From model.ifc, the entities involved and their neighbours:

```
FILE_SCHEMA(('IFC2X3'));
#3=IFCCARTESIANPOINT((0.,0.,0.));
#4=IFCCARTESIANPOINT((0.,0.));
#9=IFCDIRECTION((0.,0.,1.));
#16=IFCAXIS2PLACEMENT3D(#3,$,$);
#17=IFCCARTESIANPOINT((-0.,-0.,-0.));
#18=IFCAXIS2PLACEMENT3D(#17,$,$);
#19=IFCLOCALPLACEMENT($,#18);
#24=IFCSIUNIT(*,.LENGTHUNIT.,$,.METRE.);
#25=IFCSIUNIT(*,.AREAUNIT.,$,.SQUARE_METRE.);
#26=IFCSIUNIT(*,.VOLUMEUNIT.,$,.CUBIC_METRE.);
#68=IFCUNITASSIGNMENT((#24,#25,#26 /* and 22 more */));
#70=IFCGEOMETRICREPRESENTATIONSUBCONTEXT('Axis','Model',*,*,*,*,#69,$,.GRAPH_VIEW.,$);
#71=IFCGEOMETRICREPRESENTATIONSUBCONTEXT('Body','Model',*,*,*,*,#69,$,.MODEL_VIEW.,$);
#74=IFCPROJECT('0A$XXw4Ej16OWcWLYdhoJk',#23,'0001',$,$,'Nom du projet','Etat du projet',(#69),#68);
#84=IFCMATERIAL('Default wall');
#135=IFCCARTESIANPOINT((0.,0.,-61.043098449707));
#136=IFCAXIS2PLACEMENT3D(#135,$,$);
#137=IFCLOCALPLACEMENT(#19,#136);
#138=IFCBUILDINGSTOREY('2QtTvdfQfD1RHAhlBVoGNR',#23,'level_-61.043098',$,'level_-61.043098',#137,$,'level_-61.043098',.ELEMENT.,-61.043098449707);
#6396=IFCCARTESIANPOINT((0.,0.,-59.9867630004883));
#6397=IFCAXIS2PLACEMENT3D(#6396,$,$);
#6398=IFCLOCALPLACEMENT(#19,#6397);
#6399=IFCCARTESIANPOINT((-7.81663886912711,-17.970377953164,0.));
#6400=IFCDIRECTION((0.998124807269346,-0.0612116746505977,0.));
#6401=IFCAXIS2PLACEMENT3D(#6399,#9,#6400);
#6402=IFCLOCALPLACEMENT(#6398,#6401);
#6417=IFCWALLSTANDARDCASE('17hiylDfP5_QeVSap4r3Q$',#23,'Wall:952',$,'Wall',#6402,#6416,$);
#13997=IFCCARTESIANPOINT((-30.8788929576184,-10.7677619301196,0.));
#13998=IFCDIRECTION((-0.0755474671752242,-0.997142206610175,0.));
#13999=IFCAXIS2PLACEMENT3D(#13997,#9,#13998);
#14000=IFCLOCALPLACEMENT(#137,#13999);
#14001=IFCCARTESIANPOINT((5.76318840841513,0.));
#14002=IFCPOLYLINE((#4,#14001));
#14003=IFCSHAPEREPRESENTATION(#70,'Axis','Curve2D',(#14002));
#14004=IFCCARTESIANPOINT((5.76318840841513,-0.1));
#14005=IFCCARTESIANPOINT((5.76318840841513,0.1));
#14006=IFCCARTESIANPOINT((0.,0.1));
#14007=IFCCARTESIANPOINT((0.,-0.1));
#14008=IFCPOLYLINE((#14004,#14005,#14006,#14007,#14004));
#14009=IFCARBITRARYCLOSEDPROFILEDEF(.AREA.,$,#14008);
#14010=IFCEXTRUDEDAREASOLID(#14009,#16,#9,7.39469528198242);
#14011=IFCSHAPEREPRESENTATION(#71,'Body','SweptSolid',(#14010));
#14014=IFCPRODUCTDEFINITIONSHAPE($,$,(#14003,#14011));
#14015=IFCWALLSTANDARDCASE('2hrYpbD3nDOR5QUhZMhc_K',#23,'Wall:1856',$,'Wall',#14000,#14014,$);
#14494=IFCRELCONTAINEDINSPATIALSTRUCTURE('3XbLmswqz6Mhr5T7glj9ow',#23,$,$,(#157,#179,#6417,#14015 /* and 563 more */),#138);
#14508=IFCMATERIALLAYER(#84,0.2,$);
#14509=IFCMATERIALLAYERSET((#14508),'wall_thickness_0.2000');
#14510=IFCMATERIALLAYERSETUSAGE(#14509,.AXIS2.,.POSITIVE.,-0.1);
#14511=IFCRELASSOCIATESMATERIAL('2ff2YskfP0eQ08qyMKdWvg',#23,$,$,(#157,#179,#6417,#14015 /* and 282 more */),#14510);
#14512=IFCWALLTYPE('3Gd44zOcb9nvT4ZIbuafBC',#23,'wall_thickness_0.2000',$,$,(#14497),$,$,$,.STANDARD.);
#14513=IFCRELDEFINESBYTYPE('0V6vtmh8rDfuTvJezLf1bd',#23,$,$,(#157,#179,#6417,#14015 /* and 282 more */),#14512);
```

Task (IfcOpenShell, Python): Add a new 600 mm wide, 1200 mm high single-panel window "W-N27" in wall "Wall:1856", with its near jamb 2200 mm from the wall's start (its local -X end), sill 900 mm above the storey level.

```python
import numpy as np
import ifcopenshell
import ifcopenshell.api.feature
import ifcopenshell.api.geometry
import ifcopenshell.api.root
import ifcopenshell.api.spatial
import ifcopenshell.api.type
import ifcopenshell.geom
import ifcopenshell.util.element
import ifcopenshell.util.placement
import ifcopenshell.util.representation
import ifcopenshell.util.shape
import ifcopenshell.util.unit

model = ifcopenshell.open("model.ifc")
unit_scale = ifcopenshell.util.unit.calculate_unit_scale(model)
settings = ifcopenshell.geom.settings()


def volume(element):
    """Net volume in cubic metres, openings subtracted."""
    shape = ifcopenshell.geom.create_shape(settings, element)
    return ifcopenshell.util.shape.get_volume(shape.geometry)


wall = model.by_guid("2hrYpbD3nDOR5QUhZMhc_K")
storey = ifcopenshell.util.element.get_container(wall, ifc_class="IfcBuildingStorey")
context = ifcopenshell.util.representation.get_context(model, "Model", "Body", "MODEL_VIEW")
before = volume(wall)

width, height, from_end, sill = 0.6, 1.2, 2.2, 0.9  # metres

# The wall runs along its own X axis, and the end named is its -X end.
wall_shape = ifcopenshell.geom.create_shape(settings, wall)
x, y, z = ifcopenshell.util.shape.get_vertices(wall_shape.geometry).T
start = x.min() + from_end
face, thickness = float(y.min()), float(y.max() - y.min())
wall_matrix = ifcopenshell.util.placement.get_local_placement(wall.ObjectPlacement)
level = ifcopenshell.util.placement.get_local_placement(storey.ObjectPlacement)[2, 3]


def in_wall(x, y):
    """Placement at x, y metres in the wall's axes, at sill height."""
    matrix = wall_matrix.copy()
    matrix[:, 3] = wall_matrix @ np.array([x / unit_scale, y / unit_scale, 0.0, 1.0])
    matrix[2, 3] = level + sill / unit_scale
    return matrix


# Opening: a box that overshoots both wall faces by 50 mm.
opening = ifcopenshell.api.root.create_entity(model, ifc_class="IfcOpeningElement")
box = ifcopenshell.api.geometry.add_wall_representation(
    model, context=context, length=width, height=height, thickness=thickness + 0.1
)
ifcopenshell.api.geometry.assign_representation(model, product=opening, representation=box)
ifcopenshell.api.geometry.edit_object_placement(model, product=opening, matrix=in_wall(start, face - 0.05), is_si=False)
ifcopenshell.api.feature.add_feature(model, feature=opening, element=wall)

window = ifcopenshell.api.root.create_entity(model, ifc_class="IfcWindow", name="W-N27")
window.OverallWidth, window.OverallHeight = width / unit_scale, height / unit_scale
body = ifcopenshell.api.geometry.add_window_representation(
    model,
    context=context,
    overall_width=window.OverallWidth,
    overall_height=window.OverallHeight,
    partition_type="SINGLE_PANEL",
)
ifcopenshell.api.geometry.assign_representation(model, product=window, representation=body)
ifcopenshell.api.spatial.assign_container(model, products=[window], relating_structure=storey)
fills = ifcopenshell.api.feature.add_filling(model, opening=opening, element=window)
fills.OwnerHistory = window.OwnerHistory  # required in IFC2X3

# IFC2X3 keeps the operation on the window style.
style = ifcopenshell.api.root.create_entity(model, ifc_class="IfcWindowStyle", name="W-N27")
style.OperationType, style.ConstructionType = "SINGLE_PANEL", "NOTDEFINED"
style.ParameterTakesPrecedence = style.Sizeable = False
ifcopenshell.api.type.assign_type(model, related_objects=[window], relating_type=style)

# Centre the window in the wall's thickness.
ifcopenshell.api.geometry.edit_object_placement(model, product=window, matrix=in_wall(start, face), is_si=False)
window_shape = ifcopenshell.geom.create_shape(settings, window)
depth = ifcopenshell.util.shape.get_vertices(window_shape.geometry)[:, 1]
offset = face + thickness / 2 - (depth.min() + depth.max()) / 2
ifcopenshell.api.geometry.edit_object_placement(model, product=window, matrix=in_wall(start, offset), is_si=False)

after = volume(wall)

print(f"wall volume {before:.3f} -> {after:.3f} m3")

model.write("model_edited.ifc")
```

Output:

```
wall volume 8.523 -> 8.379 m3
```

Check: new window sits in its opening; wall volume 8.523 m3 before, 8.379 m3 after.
